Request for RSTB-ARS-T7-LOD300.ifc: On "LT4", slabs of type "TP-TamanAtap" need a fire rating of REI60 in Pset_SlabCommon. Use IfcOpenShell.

First a look at what the model holds.

```python
import ifcopenshell
import ifcopenshell.util.element

model = ifcopenshell.open("RSTB-ARS-T7-LOD300.ifc")
print(model.schema)
storey = next(s for s in model.by_type("IfcBuildingStorey") if s.Name == "LT4")
slabs = [e for e in ifcopenshell.util.element.get_decomposition(storey) if e.is_a("IfcSlab")]
seen = {}
for e in slabs:
    element_type = ifcopenshell.util.element.get_type(e)
    key = (element_type.Name if element_type != e and element_type else None, ifcopenshell.util.element.get_pset(e, "Pset_SlabCommon", "FireRating"))
    seen[key] = seen.get(key, 0) + 1
for (name, value), count in sorted(seen.items(), key=str):
    print(count, "x", name, "|", value)
```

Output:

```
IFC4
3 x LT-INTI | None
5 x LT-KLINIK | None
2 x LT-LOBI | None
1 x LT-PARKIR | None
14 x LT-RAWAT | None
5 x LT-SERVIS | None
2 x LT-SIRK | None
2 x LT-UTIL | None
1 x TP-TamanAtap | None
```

```python
import ifcopenshell
import ifcopenshell.api.pset
import ifcopenshell.util.element

model = ifcopenshell.open("RSTB-ARS-T7-LOD300.ifc")

storey = next(s for s in model.by_type("IfcBuildingStorey") if s.Name == "LT4")
slabs = [e for e in ifcopenshell.util.element.get_decomposition(storey) if e.is_a("IfcSlab")]

count = 0
for e in slabs:
    element_type = ifcopenshell.util.element.get_type(e)
    if element_type in (None, e) or element_type.Name != "TP-TamanAtap":
        continue
    # add_pset returns the element's existing set when there is one.
    pset = ifcopenshell.api.pset.add_pset(model, product=e, name="Pset_SlabCommon")
    ifcopenshell.api.pset.edit_pset(model, pset=pset, properties={"FireRating": "REI60"})
    count += 1

print(count, "slabs updated")

model.write("RSTB-ARS-T7-LOD300_rev.ifc")
```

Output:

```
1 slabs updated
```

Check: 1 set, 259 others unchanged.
